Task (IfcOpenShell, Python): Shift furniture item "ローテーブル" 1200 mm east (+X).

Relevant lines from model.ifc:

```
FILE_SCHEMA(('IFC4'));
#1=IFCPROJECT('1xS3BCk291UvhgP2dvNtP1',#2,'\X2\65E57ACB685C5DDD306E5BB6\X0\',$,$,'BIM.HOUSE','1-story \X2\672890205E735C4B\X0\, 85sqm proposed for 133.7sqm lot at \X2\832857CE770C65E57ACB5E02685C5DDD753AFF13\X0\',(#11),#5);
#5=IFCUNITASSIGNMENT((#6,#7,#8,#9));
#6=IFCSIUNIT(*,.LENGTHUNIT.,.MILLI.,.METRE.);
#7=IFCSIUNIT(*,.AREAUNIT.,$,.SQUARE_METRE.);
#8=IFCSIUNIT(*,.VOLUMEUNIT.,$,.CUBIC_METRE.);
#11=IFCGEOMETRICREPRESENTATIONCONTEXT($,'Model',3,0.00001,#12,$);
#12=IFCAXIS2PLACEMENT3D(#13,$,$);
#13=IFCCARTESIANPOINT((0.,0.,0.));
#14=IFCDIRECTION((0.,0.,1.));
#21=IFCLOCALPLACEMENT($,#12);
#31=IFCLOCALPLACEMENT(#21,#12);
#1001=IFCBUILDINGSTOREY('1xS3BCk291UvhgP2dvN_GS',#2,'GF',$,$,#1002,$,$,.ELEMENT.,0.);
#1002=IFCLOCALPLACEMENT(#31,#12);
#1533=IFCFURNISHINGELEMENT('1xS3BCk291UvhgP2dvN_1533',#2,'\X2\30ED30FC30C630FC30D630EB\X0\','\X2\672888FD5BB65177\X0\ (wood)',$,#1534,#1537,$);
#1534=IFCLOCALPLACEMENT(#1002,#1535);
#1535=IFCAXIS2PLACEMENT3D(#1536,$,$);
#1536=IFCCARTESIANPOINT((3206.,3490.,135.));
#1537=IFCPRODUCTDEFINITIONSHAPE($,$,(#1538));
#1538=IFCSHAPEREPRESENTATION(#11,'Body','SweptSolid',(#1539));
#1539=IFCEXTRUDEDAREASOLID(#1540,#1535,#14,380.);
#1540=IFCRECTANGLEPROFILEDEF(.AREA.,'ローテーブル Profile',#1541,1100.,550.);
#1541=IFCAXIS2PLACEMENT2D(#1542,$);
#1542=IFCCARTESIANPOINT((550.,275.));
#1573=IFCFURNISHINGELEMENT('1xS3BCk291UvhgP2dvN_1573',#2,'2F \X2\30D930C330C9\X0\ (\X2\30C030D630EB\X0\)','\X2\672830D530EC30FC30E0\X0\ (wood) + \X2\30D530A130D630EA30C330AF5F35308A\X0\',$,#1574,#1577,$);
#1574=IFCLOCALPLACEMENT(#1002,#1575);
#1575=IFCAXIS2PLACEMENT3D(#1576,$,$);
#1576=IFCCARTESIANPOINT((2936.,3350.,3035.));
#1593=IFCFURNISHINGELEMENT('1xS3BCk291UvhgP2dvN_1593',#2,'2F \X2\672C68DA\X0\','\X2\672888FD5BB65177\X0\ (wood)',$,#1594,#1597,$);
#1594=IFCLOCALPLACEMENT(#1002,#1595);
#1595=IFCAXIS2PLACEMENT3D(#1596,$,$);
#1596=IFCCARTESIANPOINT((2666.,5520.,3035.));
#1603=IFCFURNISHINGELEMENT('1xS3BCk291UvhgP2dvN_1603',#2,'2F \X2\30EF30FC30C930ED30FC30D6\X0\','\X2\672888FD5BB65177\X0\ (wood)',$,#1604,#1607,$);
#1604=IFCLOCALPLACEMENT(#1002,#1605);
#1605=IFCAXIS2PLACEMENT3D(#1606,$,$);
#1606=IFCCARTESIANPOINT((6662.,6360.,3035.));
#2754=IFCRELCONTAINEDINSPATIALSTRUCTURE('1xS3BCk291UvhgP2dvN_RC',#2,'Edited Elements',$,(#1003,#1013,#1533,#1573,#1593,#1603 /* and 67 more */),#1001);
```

```python
import ifcopenshell
import ifcopenshell.api.geometry
import ifcopenshell.util.placement

model = ifcopenshell.open("model.ifc")

item = model.by_id(1533)
matrix = ifcopenshell.util.placement.get_local_placement(item.ObjectPlacement)
matrix[0, 3] += 1200.0
ifcopenshell.api.geometry.edit_object_placement(model, product=item, matrix=matrix, is_si=False)

print(ifcopenshell.util.placement.get_local_placement(item.ObjectPlacement).round(3) + 0.0)

model.write("model_v2.ifc")
```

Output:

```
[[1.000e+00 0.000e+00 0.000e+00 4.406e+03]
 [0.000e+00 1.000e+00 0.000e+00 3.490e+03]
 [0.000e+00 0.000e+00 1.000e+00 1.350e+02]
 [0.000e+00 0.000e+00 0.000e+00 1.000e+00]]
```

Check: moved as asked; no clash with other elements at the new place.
